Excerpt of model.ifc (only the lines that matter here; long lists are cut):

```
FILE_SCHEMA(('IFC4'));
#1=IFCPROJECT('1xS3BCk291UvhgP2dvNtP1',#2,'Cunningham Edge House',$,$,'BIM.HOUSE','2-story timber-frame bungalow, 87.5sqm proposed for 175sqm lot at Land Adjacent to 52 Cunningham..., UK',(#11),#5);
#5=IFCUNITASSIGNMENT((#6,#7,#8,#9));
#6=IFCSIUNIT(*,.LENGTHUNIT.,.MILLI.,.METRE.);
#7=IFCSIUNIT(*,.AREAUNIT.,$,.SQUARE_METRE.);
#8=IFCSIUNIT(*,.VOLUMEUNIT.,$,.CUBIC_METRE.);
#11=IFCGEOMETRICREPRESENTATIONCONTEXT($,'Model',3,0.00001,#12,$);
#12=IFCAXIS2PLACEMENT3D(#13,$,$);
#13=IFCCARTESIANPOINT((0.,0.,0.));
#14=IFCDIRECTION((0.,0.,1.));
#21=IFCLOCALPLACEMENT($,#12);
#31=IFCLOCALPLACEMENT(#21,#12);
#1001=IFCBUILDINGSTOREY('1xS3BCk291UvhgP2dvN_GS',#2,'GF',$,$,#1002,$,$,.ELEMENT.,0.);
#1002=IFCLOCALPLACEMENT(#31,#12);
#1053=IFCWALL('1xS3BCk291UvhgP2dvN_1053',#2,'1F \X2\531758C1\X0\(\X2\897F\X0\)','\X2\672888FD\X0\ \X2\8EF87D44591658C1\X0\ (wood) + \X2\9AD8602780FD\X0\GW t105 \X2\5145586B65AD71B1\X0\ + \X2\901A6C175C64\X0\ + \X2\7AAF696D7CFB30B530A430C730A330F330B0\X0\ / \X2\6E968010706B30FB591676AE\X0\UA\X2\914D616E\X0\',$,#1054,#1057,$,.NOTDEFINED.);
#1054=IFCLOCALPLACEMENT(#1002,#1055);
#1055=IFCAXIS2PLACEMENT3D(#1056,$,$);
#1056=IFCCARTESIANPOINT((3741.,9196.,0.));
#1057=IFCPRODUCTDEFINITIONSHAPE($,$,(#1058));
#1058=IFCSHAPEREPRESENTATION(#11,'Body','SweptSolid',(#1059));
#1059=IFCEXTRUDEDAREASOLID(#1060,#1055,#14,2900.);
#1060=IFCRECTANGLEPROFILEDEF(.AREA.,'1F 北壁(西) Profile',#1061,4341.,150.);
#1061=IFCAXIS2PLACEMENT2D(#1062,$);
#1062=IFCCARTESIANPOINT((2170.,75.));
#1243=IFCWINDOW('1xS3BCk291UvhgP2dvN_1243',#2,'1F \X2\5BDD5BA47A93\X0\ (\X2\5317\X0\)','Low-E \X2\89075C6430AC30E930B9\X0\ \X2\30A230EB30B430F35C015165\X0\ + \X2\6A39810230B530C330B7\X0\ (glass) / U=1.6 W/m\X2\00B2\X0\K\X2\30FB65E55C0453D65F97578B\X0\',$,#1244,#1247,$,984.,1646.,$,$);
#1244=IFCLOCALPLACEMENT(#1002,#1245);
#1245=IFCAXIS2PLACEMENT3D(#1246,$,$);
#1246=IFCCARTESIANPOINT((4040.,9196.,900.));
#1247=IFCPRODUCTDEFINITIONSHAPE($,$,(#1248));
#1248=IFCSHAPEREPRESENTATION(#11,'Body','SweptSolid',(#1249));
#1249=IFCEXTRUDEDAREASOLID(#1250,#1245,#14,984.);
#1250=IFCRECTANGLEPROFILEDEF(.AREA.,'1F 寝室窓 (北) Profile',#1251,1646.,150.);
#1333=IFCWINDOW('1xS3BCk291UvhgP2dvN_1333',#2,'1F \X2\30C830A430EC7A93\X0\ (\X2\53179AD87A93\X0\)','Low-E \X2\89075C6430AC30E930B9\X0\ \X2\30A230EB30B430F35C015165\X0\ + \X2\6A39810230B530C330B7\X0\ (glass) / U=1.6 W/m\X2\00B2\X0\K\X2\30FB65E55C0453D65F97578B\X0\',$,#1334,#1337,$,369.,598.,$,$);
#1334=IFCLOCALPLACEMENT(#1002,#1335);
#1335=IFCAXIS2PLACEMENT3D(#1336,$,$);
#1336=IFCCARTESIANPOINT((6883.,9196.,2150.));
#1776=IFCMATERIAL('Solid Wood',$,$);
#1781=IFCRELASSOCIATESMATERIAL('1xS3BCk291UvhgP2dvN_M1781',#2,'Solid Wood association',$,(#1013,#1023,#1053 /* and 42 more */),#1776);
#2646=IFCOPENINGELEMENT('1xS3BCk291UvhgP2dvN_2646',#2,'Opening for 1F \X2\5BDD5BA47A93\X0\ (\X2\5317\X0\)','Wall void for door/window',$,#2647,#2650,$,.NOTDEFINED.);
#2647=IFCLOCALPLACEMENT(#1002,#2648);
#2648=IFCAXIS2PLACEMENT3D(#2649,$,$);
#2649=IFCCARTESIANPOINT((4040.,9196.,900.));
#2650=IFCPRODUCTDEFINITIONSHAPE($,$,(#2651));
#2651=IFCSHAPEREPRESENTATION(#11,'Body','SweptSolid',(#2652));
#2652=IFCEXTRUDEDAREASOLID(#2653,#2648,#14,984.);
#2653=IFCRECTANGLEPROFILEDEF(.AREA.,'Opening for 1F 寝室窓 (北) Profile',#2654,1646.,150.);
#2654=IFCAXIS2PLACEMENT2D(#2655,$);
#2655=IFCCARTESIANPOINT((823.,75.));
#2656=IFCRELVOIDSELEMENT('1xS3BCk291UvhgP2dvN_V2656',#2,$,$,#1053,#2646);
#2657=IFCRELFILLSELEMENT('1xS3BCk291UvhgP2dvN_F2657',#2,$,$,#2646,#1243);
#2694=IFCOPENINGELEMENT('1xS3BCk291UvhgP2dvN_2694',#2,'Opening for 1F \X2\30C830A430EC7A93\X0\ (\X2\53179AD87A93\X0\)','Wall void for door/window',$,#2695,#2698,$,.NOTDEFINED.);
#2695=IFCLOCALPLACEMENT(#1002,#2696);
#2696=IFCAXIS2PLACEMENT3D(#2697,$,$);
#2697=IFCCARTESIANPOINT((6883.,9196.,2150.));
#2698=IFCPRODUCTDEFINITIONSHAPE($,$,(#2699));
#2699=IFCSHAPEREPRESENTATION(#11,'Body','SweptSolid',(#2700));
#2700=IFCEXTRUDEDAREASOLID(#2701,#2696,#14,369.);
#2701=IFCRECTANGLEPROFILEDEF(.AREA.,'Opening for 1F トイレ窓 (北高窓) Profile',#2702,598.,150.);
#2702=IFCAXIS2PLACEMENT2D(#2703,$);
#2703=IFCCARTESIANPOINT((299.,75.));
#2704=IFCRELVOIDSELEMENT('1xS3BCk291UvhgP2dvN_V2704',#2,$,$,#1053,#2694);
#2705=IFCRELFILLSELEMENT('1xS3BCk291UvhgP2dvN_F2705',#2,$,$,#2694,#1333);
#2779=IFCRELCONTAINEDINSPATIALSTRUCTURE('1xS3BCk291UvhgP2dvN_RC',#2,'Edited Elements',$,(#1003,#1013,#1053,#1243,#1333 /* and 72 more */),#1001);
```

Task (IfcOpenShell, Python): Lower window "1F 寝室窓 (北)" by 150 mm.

```python
import numpy as np
import ifcopenshell
import ifcopenshell.api.geometry
import ifcopenshell.util.placement
import ifcopenshell.util.unit

model = ifcopenshell.open("model.ifc")
unit_scale = ifcopenshell.util.unit.calculate_unit_scale(model)

window = model.by_guid("1xS3BCk291UvhgP2dvN_1243")
opening = window.FillsVoids[0].RelatingOpeningElement
dz = -150.0

shift = np.array([0.0, 0.0, dz])
# The window is not placed relative to its opening, so move both.
for product in (opening, window):
    matrix = ifcopenshell.util.placement.get_local_placement(product.ObjectPlacement)
    matrix[:3, 3] += shift
    ifcopenshell.api.geometry.edit_object_placement(model, product=product, matrix=matrix, is_si=False)

print(f"moved by {dz * unit_scale:+.3f} m")

model.write("model_rev.ifc")
```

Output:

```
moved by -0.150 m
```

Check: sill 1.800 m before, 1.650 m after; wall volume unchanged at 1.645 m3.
